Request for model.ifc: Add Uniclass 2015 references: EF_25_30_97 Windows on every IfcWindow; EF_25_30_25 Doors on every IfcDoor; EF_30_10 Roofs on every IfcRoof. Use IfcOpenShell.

First a look at what the model holds.

```python
import ifcopenshell

model = ifcopenshell.open("model.ifc")
print(model.schema)
print("classifications:", [c.Name for c in model.by_type("IfcClassification")])
for ifc_class in ("IfcDoor", "IfcRoof", "IfcStair", "IfcWall", "IfcWindow"):
    print(ifc_class, len(model.by_type(ifc_class)))
```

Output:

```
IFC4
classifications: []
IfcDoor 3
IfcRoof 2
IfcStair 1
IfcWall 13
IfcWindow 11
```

```python
import ifcopenshell
import ifcopenshell.api.classification

model = ifcopenshell.open("model.ifc")

system = ifcopenshell.api.classification.add_classification(model, classification="Uniclass 2015")

codes = {
    "IfcWindow": ("EF_25_30_97", "Windows"),
    "IfcDoor": ("EF_25_30_25", "Doors"),
    "IfcRoof": ("EF_30_10", "Roofs"),
}
for ifc_class, (code, name) in codes.items():
    products = model.by_type(ifc_class)
    ifcopenshell.api.classification.add_reference(
        model, products=products, classification=system, identification=code, name=name
    )
    print(code, len(products))

model.write("model-out.ifc")
```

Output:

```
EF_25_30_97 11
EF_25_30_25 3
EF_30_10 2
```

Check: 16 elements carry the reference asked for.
